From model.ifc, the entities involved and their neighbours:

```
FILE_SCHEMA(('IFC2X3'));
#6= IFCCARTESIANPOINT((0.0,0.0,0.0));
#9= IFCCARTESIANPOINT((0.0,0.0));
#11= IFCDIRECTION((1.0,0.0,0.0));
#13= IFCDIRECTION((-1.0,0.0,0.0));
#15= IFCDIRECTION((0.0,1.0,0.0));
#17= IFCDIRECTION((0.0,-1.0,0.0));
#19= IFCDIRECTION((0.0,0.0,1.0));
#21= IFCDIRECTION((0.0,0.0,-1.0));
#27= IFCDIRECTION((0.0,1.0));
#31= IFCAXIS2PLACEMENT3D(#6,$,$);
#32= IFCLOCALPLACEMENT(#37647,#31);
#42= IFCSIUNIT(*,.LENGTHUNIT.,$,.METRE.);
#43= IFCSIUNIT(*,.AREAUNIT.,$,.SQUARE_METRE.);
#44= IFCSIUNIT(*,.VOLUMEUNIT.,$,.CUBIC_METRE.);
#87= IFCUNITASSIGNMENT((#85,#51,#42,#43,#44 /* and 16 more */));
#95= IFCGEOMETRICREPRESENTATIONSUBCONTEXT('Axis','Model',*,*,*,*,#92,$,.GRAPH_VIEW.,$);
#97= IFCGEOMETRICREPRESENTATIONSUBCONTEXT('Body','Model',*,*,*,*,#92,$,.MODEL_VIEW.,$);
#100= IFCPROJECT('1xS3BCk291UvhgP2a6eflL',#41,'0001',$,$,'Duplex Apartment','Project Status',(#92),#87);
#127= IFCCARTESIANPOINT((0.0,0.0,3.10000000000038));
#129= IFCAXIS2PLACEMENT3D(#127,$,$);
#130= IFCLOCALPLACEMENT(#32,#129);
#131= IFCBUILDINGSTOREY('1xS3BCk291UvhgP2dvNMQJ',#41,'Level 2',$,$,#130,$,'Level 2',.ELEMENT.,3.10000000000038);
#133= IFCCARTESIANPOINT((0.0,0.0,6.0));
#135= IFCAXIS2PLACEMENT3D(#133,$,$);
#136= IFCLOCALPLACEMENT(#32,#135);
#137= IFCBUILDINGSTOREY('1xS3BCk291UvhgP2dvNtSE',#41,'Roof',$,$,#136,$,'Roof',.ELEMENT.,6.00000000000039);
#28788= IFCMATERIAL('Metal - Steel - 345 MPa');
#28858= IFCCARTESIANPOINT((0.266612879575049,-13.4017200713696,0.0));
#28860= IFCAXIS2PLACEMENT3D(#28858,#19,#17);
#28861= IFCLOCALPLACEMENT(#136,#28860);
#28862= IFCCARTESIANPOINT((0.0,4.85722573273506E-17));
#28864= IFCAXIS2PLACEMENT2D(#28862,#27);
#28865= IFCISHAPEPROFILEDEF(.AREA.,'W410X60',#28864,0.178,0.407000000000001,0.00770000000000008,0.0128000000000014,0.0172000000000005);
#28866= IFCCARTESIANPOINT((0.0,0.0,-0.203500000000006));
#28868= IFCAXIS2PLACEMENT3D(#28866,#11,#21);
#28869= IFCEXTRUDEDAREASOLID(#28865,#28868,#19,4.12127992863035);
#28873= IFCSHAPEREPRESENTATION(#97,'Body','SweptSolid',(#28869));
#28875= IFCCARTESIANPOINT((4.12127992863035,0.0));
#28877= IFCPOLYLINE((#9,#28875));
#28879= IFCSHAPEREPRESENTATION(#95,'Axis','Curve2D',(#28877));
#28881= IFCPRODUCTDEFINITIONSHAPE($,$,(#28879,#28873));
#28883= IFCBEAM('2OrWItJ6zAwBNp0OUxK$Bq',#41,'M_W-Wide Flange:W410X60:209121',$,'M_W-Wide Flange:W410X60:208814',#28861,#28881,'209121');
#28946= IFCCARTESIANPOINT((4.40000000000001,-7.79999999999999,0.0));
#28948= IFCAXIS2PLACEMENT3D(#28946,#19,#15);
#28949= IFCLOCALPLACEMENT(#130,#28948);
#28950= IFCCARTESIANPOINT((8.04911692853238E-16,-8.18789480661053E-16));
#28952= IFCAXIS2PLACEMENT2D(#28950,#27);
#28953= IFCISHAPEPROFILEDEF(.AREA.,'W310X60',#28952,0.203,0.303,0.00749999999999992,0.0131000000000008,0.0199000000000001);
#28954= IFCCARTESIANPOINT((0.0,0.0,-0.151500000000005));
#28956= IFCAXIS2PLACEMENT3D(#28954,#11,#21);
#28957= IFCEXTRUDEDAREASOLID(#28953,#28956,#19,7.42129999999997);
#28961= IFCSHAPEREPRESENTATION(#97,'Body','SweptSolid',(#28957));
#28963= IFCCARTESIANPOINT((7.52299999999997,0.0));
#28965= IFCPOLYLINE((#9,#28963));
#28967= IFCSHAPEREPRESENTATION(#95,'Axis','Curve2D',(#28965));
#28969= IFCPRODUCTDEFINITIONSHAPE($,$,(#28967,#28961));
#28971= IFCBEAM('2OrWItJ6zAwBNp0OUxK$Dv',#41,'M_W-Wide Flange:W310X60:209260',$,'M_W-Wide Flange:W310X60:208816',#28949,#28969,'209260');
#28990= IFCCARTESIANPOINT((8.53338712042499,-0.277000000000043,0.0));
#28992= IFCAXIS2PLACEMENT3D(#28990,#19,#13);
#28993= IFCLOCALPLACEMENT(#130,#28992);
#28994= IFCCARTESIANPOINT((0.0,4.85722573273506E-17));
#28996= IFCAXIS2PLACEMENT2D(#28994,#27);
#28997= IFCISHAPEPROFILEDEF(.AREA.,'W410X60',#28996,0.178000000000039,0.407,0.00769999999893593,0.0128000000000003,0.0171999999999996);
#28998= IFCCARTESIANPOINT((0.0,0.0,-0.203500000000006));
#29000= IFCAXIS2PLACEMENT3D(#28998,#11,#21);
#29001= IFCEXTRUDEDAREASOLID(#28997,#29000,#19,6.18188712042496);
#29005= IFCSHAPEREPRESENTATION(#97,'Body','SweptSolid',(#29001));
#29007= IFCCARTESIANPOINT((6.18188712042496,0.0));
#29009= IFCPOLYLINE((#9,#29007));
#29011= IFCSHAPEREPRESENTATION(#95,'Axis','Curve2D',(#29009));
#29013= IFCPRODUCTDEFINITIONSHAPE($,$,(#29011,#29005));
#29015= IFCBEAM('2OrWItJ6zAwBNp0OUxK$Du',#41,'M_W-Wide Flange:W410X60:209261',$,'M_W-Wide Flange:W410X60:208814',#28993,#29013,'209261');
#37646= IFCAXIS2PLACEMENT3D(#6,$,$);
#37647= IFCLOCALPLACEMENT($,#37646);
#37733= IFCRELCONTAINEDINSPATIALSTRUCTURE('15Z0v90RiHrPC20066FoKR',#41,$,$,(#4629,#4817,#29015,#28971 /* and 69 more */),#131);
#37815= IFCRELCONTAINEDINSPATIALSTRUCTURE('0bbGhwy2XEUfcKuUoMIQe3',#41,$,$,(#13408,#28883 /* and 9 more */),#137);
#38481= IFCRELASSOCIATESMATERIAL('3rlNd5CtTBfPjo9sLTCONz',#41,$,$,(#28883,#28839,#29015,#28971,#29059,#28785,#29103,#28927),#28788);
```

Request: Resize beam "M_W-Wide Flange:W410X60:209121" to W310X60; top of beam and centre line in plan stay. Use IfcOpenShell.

```python
import ifcopenshell
import ifcopenshell.util.element
import ifcopenshell.util.representation

model = ifcopenshell.open("model.ifc")

member = model.by_guid("2OrWItJ6zAwBNp0OUxK$Bq")
source = next(p for p in model.by_type("IfcIShapeProfileDef") if p.ProfileName == "W310X60")

body = ifcopenshell.util.representation.get_representation(member, "Model", "Body")
solid = body.Items[0]
old_profile = solid.SweptArea

# Copy the section's sizes but keep this member's own profile position.
profile = ifcopenshell.util.element.copy(model, source)
# Profiles are centred, so shift by half the change in depth to hold the top.
shift = (old_profile.OverallDepth - profile.OverallDepth) / 2
x, y = old_profile.Position.Location.Coordinates
up = (-1.0, 0.0)  # upwards, in the solid's own plane
location = model.createIfcCartesianPoint((x + up[0] * shift, y + up[1] * shift))
profile.Position = model.createIfcAxis2Placement2D(location, old_profile.Position.RefDirection)
solid.SweptArea = profile
if not model.get_total_inverses(old_profile):
    ifcopenshell.util.element.remove_deep2(model, old_profile)
member.Name = member.Name.replace("W410X60", "W310X60")
member.ObjectType = member.ObjectType.replace("W410X60", "W310X60")

print(solid.SweptArea)

model.write("model_rev.ifc")
```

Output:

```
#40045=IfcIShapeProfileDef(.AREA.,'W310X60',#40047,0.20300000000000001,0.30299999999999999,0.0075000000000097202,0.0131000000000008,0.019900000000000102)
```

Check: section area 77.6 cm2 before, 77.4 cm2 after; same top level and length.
